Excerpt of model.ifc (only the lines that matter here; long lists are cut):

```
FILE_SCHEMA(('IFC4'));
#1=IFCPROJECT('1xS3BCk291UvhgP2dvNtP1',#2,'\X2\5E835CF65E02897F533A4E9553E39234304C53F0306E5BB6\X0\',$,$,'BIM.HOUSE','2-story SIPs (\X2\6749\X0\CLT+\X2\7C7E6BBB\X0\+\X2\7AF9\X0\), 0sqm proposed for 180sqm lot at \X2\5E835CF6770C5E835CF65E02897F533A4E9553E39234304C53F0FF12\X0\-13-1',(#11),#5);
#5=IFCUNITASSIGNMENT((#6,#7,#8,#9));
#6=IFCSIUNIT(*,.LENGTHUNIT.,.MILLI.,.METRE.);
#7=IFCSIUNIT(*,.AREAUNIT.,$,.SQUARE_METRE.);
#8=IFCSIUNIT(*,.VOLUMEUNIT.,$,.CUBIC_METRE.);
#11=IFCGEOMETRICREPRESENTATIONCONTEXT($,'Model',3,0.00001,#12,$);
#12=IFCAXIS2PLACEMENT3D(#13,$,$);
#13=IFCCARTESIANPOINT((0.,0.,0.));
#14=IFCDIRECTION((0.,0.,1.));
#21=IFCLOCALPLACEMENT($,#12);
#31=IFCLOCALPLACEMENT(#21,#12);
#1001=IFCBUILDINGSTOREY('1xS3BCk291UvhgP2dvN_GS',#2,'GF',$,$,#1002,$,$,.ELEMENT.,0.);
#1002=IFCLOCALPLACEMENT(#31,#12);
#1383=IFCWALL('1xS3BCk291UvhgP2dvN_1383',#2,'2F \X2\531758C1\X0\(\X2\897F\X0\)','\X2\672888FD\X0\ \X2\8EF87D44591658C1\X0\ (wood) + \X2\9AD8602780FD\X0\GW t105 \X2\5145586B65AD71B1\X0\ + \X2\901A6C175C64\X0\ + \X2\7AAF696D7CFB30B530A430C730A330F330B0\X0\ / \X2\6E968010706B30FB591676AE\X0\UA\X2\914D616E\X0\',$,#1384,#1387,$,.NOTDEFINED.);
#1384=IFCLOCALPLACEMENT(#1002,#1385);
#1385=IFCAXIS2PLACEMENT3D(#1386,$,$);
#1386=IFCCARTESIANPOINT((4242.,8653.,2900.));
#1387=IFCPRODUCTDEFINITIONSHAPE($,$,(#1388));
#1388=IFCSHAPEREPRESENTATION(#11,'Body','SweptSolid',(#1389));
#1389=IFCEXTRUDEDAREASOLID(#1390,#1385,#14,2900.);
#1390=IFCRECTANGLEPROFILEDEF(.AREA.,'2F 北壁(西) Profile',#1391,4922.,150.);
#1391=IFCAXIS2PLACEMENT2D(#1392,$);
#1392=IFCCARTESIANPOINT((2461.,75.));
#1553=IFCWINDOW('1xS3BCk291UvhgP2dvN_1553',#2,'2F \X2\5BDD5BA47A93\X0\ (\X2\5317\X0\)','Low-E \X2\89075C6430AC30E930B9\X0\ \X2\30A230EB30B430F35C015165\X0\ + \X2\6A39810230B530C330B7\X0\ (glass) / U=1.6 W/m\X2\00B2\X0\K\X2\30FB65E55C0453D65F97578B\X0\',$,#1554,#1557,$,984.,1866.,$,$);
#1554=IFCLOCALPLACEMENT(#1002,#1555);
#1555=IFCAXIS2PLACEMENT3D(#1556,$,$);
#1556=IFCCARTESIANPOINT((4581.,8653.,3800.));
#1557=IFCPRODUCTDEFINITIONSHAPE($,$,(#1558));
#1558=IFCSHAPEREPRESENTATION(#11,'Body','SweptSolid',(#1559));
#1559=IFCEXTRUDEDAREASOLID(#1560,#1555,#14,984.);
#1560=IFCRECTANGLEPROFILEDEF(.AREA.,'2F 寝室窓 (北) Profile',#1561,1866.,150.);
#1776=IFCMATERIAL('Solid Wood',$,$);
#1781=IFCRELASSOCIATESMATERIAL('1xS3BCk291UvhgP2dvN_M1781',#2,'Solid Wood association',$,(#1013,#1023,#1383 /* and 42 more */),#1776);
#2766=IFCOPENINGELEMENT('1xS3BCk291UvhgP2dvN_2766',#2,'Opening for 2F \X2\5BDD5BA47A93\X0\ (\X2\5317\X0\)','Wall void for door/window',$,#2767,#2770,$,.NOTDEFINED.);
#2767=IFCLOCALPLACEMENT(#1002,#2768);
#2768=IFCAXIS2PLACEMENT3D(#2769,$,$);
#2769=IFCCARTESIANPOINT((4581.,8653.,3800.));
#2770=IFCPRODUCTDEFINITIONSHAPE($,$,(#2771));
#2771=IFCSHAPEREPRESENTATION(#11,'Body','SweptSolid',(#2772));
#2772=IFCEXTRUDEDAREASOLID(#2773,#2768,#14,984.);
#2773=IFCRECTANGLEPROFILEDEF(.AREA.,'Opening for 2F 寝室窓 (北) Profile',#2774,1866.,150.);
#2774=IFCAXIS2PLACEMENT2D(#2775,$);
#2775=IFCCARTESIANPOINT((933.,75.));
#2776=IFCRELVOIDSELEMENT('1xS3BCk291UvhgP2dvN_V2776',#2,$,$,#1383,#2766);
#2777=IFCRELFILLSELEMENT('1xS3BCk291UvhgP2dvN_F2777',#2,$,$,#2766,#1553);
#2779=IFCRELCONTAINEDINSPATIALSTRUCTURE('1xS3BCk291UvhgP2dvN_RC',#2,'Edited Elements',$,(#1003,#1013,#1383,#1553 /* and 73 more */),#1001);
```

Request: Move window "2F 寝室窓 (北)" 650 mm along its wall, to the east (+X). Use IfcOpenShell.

```python
import ifcopenshell
import ifcopenshell.api.geometry
import ifcopenshell.util.placement
import ifcopenshell.util.unit

model = ifcopenshell.open("model.ifc")
unit_scale = ifcopenshell.util.unit.calculate_unit_scale(model)

window = model.by_guid("1xS3BCk291UvhgP2dvN_1553")
opening = window.FillsVoids[0].RelatingOpeningElement
wall = opening.VoidsElements[0].RelatingBuildingElement

wall_matrix = ifcopenshell.util.placement.get_local_placement(wall.ObjectPlacement)
shift = wall_matrix[:3, 0] * 0.65 / unit_scale
before = ifcopenshell.util.placement.get_local_placement(window.ObjectPlacement)[:3, 3].copy()

# The window is not placed relative to its opening, so move both.
for product in (opening, window):
    matrix = ifcopenshell.util.placement.get_local_placement(product.ObjectPlacement)
    matrix[:3, 3] += shift
    ifcopenshell.api.geometry.edit_object_placement(model, product=product, matrix=matrix, is_si=False)

after = ifcopenshell.util.placement.get_local_placement(window.ObjectPlacement)[:3, 3]
print("window moved by", (after - before).round(3) + 0.0)

model.write("model_edited.ifc")
```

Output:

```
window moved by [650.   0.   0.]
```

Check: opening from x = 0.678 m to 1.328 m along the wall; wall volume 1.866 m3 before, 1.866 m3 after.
